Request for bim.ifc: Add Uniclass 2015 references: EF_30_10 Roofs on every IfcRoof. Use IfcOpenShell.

First a look at what the model holds.

```python
import ifcopenshell

model = ifcopenshell.open("bim.ifc")
print(model.schema)
print("classifications:", [c.Name for c in model.by_type("IfcClassification")])
for ifc_class in ("IfcDoor", "IfcRoof", "IfcStair", "IfcWall", "IfcWindow"):
    print(ifc_class, len(model.by_type(ifc_class)))
```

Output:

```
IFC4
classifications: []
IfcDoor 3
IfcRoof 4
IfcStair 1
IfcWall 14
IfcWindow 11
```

```python
import ifcopenshell
import ifcopenshell.api.classification

model = ifcopenshell.open("bim.ifc")

system = ifcopenshell.api.classification.add_classification(model, classification="Uniclass 2015")

codes = {
    "IfcRoof": ("EF_30_10", "Roofs"),
}
for ifc_class, (code, name) in codes.items():
    products = model.by_type(ifc_class)
    ifcopenshell.api.classification.add_reference(
        model, products=products, classification=system, identification=code, name=name
    )
    print(code, len(products))

model.write("bim-out.ifc")
```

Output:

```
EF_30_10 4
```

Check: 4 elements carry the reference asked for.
